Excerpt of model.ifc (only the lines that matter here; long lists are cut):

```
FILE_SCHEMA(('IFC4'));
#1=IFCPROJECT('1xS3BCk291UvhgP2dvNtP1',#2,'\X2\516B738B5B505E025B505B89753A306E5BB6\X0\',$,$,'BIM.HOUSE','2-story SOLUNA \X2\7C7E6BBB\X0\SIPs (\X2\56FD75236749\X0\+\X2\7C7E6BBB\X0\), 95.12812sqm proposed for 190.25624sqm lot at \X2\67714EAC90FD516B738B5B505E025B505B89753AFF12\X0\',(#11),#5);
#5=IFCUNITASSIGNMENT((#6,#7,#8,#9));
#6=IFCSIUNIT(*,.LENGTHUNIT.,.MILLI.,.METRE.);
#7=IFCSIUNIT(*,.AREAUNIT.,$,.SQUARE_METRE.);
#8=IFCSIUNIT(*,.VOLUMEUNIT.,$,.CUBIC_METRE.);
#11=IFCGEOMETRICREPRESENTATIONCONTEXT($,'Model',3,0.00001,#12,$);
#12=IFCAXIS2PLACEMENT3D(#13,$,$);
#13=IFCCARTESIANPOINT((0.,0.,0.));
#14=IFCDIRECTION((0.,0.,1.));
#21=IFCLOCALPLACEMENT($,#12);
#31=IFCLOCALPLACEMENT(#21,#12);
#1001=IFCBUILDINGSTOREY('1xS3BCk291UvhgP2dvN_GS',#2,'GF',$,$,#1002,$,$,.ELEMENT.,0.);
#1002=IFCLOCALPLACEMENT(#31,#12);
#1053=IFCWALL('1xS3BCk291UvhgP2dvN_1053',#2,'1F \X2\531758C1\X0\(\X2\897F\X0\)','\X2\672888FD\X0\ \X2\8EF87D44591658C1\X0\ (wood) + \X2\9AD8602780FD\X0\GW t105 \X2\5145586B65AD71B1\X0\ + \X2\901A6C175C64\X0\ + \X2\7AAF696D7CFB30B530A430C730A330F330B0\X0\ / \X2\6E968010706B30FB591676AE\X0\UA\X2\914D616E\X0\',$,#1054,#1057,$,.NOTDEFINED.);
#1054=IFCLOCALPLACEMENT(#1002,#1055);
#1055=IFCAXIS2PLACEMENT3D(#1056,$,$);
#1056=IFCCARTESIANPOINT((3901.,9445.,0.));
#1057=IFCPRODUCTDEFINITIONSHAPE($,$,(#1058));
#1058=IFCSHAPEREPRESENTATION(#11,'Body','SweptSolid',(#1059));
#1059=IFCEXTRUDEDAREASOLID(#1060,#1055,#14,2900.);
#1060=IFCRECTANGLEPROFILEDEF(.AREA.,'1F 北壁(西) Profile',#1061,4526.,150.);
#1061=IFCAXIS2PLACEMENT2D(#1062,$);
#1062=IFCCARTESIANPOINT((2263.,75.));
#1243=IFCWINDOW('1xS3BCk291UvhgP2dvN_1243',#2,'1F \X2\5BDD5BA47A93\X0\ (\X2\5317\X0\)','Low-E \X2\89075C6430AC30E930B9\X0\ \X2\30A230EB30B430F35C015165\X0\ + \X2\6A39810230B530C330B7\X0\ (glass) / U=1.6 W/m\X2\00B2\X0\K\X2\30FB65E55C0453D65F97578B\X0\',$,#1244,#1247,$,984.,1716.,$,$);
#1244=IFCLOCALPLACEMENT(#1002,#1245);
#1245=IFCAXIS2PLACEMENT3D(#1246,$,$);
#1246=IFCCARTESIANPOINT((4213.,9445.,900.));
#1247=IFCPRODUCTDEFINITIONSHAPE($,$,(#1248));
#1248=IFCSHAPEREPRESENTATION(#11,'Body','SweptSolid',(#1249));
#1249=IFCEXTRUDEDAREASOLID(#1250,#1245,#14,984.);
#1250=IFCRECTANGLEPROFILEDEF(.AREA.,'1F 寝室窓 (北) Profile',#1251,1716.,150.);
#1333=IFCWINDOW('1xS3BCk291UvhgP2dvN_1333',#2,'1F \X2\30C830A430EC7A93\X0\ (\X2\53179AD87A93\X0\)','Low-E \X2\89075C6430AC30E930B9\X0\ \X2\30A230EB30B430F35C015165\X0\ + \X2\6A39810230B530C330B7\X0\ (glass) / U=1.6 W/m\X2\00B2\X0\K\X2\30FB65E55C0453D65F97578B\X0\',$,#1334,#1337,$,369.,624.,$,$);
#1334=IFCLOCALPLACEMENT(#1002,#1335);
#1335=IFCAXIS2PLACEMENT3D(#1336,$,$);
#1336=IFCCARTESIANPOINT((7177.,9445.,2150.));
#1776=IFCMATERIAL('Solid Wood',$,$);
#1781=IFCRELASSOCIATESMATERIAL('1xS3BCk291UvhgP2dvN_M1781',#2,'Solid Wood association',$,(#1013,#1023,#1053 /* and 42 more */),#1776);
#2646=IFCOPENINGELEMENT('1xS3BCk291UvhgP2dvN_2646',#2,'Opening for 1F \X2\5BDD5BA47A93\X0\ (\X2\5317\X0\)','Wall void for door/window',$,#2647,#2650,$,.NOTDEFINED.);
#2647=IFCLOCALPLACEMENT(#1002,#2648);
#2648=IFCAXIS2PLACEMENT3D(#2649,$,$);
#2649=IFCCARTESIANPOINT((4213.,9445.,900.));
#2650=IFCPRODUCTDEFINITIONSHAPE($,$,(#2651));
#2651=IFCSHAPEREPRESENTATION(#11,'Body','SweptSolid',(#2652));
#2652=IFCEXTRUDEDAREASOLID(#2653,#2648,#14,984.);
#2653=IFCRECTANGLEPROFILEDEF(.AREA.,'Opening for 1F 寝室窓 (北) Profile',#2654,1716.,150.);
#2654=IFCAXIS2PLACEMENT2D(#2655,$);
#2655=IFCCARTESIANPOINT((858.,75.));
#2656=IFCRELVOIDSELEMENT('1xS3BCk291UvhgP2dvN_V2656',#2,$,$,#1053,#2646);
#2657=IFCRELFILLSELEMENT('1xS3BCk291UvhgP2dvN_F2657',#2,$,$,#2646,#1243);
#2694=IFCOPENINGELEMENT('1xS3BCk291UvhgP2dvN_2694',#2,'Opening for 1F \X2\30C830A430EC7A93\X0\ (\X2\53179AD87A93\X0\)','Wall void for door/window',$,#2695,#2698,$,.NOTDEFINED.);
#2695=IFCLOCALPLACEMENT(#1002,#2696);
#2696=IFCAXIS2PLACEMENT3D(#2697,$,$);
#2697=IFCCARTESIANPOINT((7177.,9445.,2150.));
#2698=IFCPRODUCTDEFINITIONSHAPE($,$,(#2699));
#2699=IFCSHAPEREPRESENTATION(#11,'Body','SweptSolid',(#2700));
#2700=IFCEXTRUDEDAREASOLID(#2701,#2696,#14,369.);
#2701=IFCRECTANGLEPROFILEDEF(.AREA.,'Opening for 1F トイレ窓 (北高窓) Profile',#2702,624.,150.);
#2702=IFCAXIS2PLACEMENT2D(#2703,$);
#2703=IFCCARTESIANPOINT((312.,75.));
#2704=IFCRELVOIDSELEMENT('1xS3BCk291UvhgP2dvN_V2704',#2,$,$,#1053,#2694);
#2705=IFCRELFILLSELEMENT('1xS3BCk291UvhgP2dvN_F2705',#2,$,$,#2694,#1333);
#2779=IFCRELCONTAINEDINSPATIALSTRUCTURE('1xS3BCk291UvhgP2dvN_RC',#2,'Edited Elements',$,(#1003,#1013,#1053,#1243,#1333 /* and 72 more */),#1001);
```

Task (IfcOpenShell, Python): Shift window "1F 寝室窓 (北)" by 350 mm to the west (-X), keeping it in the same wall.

```python
import ifcopenshell
import ifcopenshell.api.geometry
import ifcopenshell.util.placement
import ifcopenshell.util.unit

model = ifcopenshell.open("model.ifc")
unit_scale = ifcopenshell.util.unit.calculate_unit_scale(model)

window = model.by_guid("1xS3BCk291UvhgP2dvN_1243")
opening = window.FillsVoids[0].RelatingOpeningElement
wall = opening.VoidsElements[0].RelatingBuildingElement

wall_matrix = ifcopenshell.util.placement.get_local_placement(wall.ObjectPlacement)
shift = wall_matrix[:3, 0] * -0.35 / unit_scale
before = ifcopenshell.util.placement.get_local_placement(window.ObjectPlacement)[:3, 3].copy()

# The window is not placed relative to its opening, so move both.
for product in (opening, window):
    matrix = ifcopenshell.util.placement.get_local_placement(product.ObjectPlacement)
    matrix[:3, 3] += shift
    ifcopenshell.api.geometry.edit_object_placement(model, product=product, matrix=matrix, is_si=False)

after = ifcopenshell.util.placement.get_local_placement(window.ObjectPlacement)[:3, 3]
print("window moved by", (after - before).round(3) + 0.0)

model.write("model_updated.ifc")
```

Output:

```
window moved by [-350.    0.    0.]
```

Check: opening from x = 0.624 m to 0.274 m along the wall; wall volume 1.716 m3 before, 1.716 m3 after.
